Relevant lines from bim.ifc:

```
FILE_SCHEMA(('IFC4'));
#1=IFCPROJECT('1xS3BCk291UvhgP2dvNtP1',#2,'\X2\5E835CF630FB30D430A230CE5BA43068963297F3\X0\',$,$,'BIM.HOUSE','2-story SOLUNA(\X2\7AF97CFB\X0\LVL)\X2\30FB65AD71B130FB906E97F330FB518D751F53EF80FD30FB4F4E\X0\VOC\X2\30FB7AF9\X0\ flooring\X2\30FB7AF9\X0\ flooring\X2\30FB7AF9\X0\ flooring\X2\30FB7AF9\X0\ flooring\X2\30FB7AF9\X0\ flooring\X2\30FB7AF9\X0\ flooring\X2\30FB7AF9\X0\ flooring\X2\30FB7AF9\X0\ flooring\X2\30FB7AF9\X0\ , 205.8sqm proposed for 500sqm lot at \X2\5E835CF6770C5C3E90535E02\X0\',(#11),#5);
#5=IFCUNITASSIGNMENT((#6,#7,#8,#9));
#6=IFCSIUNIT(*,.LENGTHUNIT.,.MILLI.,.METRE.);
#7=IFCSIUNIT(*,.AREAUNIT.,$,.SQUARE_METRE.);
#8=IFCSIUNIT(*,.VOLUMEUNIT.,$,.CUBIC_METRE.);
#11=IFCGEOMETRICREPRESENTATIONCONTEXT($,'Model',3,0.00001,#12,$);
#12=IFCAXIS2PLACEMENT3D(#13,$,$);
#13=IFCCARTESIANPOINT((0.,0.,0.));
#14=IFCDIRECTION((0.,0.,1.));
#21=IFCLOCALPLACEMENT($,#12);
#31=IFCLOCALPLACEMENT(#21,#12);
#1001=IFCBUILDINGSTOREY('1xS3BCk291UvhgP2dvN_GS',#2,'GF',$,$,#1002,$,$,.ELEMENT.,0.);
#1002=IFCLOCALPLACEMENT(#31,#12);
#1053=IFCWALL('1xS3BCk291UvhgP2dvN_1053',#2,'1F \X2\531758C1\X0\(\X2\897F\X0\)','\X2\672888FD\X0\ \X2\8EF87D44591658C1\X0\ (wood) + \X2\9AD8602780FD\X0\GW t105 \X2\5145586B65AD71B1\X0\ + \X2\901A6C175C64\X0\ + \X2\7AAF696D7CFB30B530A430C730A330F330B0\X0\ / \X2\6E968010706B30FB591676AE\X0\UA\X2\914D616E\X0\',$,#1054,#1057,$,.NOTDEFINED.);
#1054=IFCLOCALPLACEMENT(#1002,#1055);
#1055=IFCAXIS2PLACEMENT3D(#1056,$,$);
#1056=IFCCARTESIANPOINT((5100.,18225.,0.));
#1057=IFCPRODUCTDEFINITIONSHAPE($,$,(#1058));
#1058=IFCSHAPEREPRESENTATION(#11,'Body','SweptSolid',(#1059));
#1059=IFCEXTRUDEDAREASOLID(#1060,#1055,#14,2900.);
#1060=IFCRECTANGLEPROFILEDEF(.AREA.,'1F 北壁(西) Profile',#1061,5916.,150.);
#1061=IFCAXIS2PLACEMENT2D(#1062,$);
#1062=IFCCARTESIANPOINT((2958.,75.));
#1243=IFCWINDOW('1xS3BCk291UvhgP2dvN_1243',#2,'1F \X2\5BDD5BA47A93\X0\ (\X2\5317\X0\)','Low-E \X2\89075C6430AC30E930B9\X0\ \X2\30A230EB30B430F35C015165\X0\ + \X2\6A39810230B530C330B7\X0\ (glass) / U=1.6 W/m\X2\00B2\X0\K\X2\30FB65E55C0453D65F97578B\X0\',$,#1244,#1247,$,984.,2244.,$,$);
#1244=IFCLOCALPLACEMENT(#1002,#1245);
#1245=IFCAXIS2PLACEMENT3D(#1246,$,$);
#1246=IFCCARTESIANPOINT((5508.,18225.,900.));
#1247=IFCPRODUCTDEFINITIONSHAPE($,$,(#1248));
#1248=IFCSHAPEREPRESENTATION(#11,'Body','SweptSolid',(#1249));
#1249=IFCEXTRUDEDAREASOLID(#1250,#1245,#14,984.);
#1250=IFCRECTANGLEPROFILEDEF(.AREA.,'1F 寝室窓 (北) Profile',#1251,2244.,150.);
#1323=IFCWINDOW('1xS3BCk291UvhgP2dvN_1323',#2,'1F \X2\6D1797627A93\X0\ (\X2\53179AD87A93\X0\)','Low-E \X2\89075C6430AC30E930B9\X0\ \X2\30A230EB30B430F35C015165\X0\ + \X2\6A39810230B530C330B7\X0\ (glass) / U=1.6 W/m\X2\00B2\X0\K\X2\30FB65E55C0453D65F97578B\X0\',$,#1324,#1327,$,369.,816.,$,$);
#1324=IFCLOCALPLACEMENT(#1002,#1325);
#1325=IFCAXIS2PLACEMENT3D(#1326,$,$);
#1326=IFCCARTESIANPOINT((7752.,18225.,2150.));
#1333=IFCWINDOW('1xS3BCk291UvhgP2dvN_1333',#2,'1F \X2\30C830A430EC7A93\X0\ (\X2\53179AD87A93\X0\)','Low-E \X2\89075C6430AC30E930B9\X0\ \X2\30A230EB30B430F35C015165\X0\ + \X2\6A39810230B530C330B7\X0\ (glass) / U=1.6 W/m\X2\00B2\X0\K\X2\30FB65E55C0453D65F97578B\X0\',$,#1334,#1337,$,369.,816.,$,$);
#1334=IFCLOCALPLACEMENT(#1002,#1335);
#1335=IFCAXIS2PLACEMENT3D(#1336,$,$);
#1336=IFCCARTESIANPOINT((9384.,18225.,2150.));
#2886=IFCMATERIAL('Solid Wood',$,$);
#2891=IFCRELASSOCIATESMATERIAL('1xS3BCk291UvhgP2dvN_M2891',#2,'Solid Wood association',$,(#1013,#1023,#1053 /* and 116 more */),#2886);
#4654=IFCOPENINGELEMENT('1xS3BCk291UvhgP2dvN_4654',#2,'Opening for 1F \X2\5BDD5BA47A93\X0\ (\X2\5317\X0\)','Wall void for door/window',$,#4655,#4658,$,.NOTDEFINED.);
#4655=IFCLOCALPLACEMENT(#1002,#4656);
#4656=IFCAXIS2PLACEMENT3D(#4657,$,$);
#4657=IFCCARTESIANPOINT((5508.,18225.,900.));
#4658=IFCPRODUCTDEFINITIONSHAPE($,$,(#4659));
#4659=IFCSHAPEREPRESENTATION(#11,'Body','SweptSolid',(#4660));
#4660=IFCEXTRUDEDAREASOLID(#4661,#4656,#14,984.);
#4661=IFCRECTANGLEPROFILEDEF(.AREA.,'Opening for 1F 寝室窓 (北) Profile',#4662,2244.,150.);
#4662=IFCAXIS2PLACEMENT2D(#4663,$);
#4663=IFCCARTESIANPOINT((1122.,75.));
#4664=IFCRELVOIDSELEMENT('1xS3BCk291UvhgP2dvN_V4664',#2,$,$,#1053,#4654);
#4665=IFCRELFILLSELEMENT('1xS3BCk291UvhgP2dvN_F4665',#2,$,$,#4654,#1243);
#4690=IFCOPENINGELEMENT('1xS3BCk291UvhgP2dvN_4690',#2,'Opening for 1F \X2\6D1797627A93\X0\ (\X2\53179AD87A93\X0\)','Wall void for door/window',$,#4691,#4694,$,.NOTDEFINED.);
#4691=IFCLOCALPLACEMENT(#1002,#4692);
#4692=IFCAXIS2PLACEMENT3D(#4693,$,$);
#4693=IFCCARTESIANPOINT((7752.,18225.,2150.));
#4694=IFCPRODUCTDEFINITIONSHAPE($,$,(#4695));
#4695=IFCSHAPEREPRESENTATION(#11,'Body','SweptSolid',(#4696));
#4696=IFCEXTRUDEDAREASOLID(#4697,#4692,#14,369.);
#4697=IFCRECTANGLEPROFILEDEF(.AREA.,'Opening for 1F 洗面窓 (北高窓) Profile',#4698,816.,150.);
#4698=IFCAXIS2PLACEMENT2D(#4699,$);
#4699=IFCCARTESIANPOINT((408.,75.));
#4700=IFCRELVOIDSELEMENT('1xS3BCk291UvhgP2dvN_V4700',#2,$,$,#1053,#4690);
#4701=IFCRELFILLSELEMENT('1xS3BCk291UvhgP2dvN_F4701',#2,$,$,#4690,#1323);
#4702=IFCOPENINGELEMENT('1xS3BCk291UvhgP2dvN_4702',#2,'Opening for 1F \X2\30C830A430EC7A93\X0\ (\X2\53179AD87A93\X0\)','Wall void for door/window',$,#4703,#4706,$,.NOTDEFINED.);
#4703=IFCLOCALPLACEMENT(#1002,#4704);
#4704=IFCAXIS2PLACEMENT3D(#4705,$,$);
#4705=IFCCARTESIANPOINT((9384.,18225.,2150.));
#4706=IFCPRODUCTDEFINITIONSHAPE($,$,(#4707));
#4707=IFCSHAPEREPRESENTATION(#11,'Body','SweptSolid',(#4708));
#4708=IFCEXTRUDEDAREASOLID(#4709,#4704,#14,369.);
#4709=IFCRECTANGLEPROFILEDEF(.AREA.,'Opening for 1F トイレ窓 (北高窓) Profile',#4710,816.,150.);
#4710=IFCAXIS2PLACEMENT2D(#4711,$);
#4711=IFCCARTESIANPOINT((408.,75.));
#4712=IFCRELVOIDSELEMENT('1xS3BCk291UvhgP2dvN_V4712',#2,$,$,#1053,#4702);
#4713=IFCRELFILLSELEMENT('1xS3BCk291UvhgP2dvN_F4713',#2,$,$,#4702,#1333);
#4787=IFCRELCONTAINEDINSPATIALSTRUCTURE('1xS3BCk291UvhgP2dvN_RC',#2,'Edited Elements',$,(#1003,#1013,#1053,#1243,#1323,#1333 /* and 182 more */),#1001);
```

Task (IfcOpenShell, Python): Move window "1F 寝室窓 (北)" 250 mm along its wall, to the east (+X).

```python
import ifcopenshell
import ifcopenshell.api.geometry
import ifcopenshell.util.placement

model = ifcopenshell.open("bim.ifc")

window = model.by_id(1243)
opening = window.FillsVoids[0].RelatingOpeningElement
wall = opening.VoidsElements[0].RelatingBuildingElement

wall_matrix = ifcopenshell.util.placement.get_local_placement(wall.ObjectPlacement)
shift = wall_matrix[:3, 0] * 250.0
before = ifcopenshell.util.placement.get_local_placement(window.ObjectPlacement)[:3, 3].copy()

# The window is not placed relative to its opening, so move both.
for product in (opening, window):
    matrix = ifcopenshell.util.placement.get_local_placement(product.ObjectPlacement)
    matrix[:3, 3] += shift
    ifcopenshell.api.geometry.edit_object_placement(model, product=product, matrix=matrix, is_si=False)

after = ifcopenshell.util.placement.get_local_placement(window.ObjectPlacement)[:3, 3]
print("window moved by", (after - before).round(3) + 0.0)

model.write("bim_edited.ifc")
```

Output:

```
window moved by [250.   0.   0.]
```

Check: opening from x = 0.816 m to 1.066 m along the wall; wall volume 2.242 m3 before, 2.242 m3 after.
